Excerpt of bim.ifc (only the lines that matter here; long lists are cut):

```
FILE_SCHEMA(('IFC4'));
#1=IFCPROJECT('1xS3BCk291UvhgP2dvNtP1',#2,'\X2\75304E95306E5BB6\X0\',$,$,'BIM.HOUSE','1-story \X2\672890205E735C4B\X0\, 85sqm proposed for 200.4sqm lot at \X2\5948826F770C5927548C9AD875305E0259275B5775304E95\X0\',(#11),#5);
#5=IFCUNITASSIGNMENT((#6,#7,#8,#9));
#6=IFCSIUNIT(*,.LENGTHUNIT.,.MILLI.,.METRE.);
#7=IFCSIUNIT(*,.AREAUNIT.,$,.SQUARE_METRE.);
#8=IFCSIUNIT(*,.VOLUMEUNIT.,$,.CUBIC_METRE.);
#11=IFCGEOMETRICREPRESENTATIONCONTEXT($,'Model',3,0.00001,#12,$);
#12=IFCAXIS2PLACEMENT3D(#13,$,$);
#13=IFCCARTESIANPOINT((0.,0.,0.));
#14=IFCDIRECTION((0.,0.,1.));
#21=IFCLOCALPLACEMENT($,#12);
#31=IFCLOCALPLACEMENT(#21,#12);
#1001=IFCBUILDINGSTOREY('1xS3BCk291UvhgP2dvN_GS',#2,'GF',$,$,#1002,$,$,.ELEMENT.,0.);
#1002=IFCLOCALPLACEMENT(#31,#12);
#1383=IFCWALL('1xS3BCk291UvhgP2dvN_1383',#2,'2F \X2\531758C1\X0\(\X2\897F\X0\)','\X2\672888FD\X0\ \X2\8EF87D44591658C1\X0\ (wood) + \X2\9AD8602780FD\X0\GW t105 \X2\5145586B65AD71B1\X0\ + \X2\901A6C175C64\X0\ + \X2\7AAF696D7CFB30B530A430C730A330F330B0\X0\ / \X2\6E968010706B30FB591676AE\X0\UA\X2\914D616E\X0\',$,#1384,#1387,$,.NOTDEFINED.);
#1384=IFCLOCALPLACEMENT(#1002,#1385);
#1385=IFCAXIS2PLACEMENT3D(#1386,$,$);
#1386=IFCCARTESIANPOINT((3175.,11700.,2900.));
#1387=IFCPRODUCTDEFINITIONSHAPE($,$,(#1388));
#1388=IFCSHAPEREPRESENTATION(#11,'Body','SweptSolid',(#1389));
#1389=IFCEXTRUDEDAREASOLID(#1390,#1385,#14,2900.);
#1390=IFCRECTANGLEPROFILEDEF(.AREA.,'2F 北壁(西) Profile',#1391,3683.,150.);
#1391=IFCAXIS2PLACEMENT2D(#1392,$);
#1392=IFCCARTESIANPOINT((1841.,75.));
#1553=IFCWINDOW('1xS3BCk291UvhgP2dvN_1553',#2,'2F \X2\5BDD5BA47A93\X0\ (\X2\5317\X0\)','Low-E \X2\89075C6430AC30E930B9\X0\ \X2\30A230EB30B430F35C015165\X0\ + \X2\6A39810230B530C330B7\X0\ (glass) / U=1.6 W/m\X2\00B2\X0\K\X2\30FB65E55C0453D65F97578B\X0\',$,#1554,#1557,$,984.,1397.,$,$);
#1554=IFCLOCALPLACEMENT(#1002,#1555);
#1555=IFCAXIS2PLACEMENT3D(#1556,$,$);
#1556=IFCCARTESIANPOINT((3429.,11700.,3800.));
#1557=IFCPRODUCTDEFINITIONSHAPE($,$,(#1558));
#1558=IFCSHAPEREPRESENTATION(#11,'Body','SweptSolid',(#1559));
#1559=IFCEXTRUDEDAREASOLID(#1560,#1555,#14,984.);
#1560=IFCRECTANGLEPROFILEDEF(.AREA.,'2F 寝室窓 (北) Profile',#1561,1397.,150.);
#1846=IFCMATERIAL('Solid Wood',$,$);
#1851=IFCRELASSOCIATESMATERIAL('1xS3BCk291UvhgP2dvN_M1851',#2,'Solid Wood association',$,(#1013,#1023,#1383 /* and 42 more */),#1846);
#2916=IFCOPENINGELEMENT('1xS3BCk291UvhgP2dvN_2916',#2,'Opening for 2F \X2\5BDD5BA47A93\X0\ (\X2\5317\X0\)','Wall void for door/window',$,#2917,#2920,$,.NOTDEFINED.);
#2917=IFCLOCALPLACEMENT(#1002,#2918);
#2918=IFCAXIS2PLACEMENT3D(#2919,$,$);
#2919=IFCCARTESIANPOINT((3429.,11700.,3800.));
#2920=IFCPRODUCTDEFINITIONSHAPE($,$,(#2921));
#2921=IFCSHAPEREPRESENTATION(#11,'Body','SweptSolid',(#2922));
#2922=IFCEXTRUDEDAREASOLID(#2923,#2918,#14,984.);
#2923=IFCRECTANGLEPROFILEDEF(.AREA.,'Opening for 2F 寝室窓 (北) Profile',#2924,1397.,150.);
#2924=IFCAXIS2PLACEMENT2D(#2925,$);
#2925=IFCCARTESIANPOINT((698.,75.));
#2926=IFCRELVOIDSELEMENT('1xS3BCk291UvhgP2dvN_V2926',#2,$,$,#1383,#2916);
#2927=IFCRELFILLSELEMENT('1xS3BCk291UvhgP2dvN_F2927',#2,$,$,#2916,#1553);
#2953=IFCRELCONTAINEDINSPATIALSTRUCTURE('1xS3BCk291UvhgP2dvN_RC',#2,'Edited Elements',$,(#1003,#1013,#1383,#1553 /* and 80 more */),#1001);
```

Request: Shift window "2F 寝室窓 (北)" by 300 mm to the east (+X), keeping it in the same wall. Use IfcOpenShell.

```python
import ifcopenshell
import ifcopenshell.api.geometry
import ifcopenshell.util.placement
import ifcopenshell.util.unit

model = ifcopenshell.open("bim.ifc")
unit_scale = ifcopenshell.util.unit.calculate_unit_scale(model)

window = model.by_id(1553)
opening = window.FillsVoids[0].RelatingOpeningElement
wall = opening.VoidsElements[0].RelatingBuildingElement

wall_matrix = ifcopenshell.util.placement.get_local_placement(wall.ObjectPlacement)
shift = wall_matrix[:3, 0] * 0.3 / unit_scale
before = ifcopenshell.util.placement.get_local_placement(window.ObjectPlacement)[:3, 3].copy()

# The window is not placed relative to its opening, so move both.
for product in (opening, window):
    matrix = ifcopenshell.util.placement.get_local_placement(product.ObjectPlacement)
    matrix[:3, 3] += shift
    ifcopenshell.api.geometry.edit_object_placement(model, product=product, matrix=matrix, is_si=False)

after = ifcopenshell.util.placement.get_local_placement(window.ObjectPlacement)[:3, 3]
print("window moved by", (after - before).round(3) + 0.0)

model.write("bim_edited.ifc")
```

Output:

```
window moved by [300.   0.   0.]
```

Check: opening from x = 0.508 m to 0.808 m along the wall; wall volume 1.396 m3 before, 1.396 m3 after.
